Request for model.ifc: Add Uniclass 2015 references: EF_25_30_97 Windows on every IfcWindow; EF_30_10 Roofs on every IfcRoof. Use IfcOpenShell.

First a look at what the model holds.

```python
import ifcopenshell

model = ifcopenshell.open("model.ifc")
print(model.schema)
print("classifications:", [c.Name for c in model.by_type("IfcClassification")])
for ifc_class in ("IfcDoor", "IfcRoof", "IfcStair", "IfcWall", "IfcWindow"):
    print(ifc_class, len(model.by_type(ifc_class)))
```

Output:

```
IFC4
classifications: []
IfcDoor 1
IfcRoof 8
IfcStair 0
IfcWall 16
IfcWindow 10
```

```python
import ifcopenshell
import ifcopenshell.api.classification

model = ifcopenshell.open("model.ifc")

system = ifcopenshell.api.classification.add_classification(model, classification="Uniclass 2015")

codes = {
    "IfcWindow": ("EF_25_30_97", "Windows"),
    "IfcRoof": ("EF_30_10", "Roofs"),
}
for ifc_class, (code, name) in codes.items():
    products = model.by_type(ifc_class)
    ifcopenshell.api.classification.add_reference(
        model, products=products, classification=system, identification=code, name=name
    )
    print(code, len(products))

model.write("model_v2.ifc")
```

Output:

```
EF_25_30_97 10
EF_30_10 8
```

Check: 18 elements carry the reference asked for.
